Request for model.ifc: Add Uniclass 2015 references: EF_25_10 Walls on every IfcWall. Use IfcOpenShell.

First a look at what the model holds.

```python
import ifcopenshell

model = ifcopenshell.open("model.ifc")
print(model.schema)
print("classifications:", [c.Name for c in model.by_type("IfcClassification")])
for ifc_class in ("IfcDoor", "IfcRoof", "IfcStair", "IfcWall", "IfcWindow"):
    print(ifc_class, len(model.by_type(ifc_class)))
```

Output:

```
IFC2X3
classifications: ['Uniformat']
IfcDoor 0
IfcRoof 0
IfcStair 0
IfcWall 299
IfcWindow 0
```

```python
import ifcopenshell
import ifcopenshell.api.classification

model = ifcopenshell.open("model.ifc")

# IFC2X3 requires Source and Edition and has no link from the project to the system.
system = model.create_entity("IfcClassification", Source="NBS", Edition="2015", Name="Uniclass 2015")

codes = {
    "IfcWall": ("EF_25_10", "Walls"),
}
for ifc_class, (code, name) in codes.items():
    products = model.by_type(ifc_class)
    ifcopenshell.api.classification.add_reference(
        model, products=products, classification=system, identification=code, name=name
    )
    print(code, len(products))

model.write("model_rev.ifc")
```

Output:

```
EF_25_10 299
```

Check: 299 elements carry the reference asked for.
